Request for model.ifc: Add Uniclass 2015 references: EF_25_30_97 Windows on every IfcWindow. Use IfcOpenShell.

First a look at what the model holds.

```python
import ifcopenshell

model = ifcopenshell.open("model.ifc")
print(model.schema)
print("classifications:", [c.Name for c in model.by_type("IfcClassification")])
for ifc_class in ("IfcDoor", "IfcRoof", "IfcStair", "IfcWall", "IfcWindow"):
    print(ifc_class, len(model.by_type(ifc_class)))
```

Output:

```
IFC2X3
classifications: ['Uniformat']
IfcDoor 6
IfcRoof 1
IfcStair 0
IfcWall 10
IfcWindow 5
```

```python
import ifcopenshell
import ifcopenshell.api.classification

model = ifcopenshell.open("model.ifc")

# IFC2X3 requires Source and Edition and has no link from the project to the system.
system = model.create_entity("IfcClassification", Source="NBS", Edition="2015", Name="Uniclass 2015")

codes = {
    "IfcWindow": ("EF_25_30_97", "Windows"),
}
for ifc_class, (code, name) in codes.items():
    products = model.by_type(ifc_class)
    ifcopenshell.api.classification.add_reference(
        model, products=products, classification=system, identification=code, name=name
    )
    print(code, len(products))

model.write("model_v2.ifc")
```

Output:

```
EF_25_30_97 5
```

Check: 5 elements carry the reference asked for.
